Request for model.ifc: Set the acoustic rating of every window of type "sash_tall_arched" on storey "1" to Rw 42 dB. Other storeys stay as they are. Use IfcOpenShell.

First a look at what the model holds.

```python
import ifcopenshell
import ifcopenshell.util.element

model = ifcopenshell.open("model.ifc")
print(model.schema)
storey = next(s for s in model.by_type("IfcBuildingStorey") if s.Name == "1")
windows = [e for e in ifcopenshell.util.element.get_decomposition(storey) if e.is_a("IfcWindow")]
seen = {}
for e in windows:
    element_type = ifcopenshell.util.element.get_type(e)
    key = (element_type.Name if element_type != e and element_type else None, ifcopenshell.util.element.get_pset(e, "Pset_WindowCommon", "AcousticRating"))
    seen[key] = seen.get(key, 0) + 1
for (name, value), count in sorted(seen.items(), key=str):
    print(count, "x", name, "|", value)
```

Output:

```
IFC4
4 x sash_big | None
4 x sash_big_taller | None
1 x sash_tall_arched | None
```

```python
import ifcopenshell
import ifcopenshell.api.pset
import ifcopenshell.util.element

model = ifcopenshell.open("model.ifc")

storey = next(s for s in model.by_type("IfcBuildingStorey") if s.Name == "1")
windows = [e for e in ifcopenshell.util.element.get_decomposition(storey) if e.is_a("IfcWindow")]

count = 0
for e in windows:
    element_type = ifcopenshell.util.element.get_type(e)
    if element_type in (None, e) or element_type.Name != "sash_tall_arched":
        continue
    # add_pset returns the element's existing set when there is one.
    pset = ifcopenshell.api.pset.add_pset(model, product=e, name="Pset_WindowCommon")
    ifcopenshell.api.pset.edit_pset(model, pset=pset, properties={"AcousticRating": "Rw 42 dB"})
    count += 1

print(count, "windows updated")

model.write("model_v2.ifc")
```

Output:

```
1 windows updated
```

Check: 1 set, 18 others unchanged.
